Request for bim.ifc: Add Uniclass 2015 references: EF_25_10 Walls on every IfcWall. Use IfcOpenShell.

First a look at what the model holds.

```python
import ifcopenshell

model = ifcopenshell.open("bim.ifc")
print(model.schema)
print("classifications:", [c.Name for c in model.by_type("IfcClassification")])
for ifc_class in ("IfcDoor", "IfcRoof", "IfcStair", "IfcWall", "IfcWindow"):
    print(ifc_class, len(model.by_type(ifc_class)))
```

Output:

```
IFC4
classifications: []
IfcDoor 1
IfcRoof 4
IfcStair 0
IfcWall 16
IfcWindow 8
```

```python
import ifcopenshell
import ifcopenshell.api.classification

model = ifcopenshell.open("bim.ifc")

system = ifcopenshell.api.classification.add_classification(model, classification="Uniclass 2015")

codes = {
    "IfcWall": ("EF_25_10", "Walls"),
}
for ifc_class, (code, name) in codes.items():
    products = model.by_type(ifc_class)
    ifcopenshell.api.classification.add_reference(
        model, products=products, classification=system, identification=code, name=name
    )
    print(code, len(products))

model.write("bim_v2.ifc")
```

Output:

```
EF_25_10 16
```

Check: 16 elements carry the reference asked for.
